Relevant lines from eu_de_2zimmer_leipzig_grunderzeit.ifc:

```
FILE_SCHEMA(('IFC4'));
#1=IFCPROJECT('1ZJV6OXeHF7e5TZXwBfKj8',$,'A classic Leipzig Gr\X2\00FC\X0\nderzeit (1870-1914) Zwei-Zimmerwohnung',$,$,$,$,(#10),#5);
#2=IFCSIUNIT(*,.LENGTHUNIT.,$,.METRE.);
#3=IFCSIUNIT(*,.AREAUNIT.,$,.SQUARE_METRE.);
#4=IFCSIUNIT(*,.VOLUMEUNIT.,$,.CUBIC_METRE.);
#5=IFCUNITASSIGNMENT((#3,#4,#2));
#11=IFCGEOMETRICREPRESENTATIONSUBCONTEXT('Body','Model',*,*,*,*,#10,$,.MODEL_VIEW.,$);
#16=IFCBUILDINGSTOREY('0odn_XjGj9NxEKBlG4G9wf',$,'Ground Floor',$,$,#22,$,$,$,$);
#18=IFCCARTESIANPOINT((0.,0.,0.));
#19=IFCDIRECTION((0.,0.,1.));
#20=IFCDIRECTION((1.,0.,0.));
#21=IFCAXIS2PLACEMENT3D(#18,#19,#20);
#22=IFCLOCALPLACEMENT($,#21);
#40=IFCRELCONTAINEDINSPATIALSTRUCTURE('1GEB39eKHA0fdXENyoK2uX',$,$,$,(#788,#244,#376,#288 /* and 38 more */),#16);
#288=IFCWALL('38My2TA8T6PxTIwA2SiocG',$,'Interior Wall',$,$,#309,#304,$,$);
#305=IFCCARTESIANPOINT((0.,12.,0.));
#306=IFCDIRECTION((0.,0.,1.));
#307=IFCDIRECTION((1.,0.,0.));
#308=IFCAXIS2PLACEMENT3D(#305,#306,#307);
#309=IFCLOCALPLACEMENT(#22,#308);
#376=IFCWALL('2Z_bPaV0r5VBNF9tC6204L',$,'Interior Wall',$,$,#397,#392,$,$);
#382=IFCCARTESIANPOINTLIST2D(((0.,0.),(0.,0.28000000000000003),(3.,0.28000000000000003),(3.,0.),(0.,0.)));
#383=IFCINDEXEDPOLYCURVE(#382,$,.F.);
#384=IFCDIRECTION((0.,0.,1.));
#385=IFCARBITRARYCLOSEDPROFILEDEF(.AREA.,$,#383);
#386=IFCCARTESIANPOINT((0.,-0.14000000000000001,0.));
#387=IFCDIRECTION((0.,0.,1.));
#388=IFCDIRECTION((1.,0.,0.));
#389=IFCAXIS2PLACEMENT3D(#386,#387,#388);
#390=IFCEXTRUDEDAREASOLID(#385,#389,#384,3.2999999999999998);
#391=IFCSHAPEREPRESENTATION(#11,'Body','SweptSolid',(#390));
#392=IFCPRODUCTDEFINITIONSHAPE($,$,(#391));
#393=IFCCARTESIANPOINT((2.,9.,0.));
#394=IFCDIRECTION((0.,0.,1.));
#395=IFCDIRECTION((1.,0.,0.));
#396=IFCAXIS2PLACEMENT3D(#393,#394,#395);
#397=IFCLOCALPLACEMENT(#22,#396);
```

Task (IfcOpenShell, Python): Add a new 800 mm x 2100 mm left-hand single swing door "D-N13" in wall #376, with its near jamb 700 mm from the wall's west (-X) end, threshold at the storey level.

```python
import numpy as np
import ifcopenshell
import ifcopenshell.api.feature
import ifcopenshell.api.geometry
import ifcopenshell.api.root
import ifcopenshell.api.spatial
import ifcopenshell.geom
import ifcopenshell.util.element
import ifcopenshell.util.placement
import ifcopenshell.util.representation
import ifcopenshell.util.shape
import ifcopenshell.util.unit

model = ifcopenshell.open("eu_de_2zimmer_leipzig_grunderzeit.ifc")
unit_scale = ifcopenshell.util.unit.calculate_unit_scale(model)
settings = ifcopenshell.geom.settings()


def volume(element):
    """Net volume in cubic metres, openings subtracted."""
    shape = ifcopenshell.geom.create_shape(settings, element)
    return ifcopenshell.util.shape.get_volume(shape.geometry)


wall = model.by_guid("2Z_bPaV0r5VBNF9tC6204L")
storey = ifcopenshell.util.element.get_container(wall, ifc_class="IfcBuildingStorey")
context = ifcopenshell.util.representation.get_context(model, "Model", "Body", "MODEL_VIEW")
before = volume(wall)

width, height, from_end, sill = 0.8, 2.1, 0.7, 0.0  # metres

# The wall runs along its own X axis, and the end named is its -X end.
wall_shape = ifcopenshell.geom.create_shape(settings, wall)
x, y, z = ifcopenshell.util.shape.get_vertices(wall_shape.geometry).T
start = x.min() + from_end
face, thickness = float(y.min()), float(y.max() - y.min())
wall_matrix = ifcopenshell.util.placement.get_local_placement(wall.ObjectPlacement)
level = ifcopenshell.util.placement.get_local_placement(storey.ObjectPlacement)[2, 3]


def in_wall(x, y):
    """Placement at x, y metres in the wall's axes, at sill height."""
    matrix = wall_matrix.copy()
    matrix[:, 3] = wall_matrix @ np.array([x / unit_scale, y / unit_scale, 0.0, 1.0])
    matrix[2, 3] = level + sill / unit_scale
    return matrix


# Opening: a box that overshoots both wall faces by 50 mm.
opening = ifcopenshell.api.root.create_entity(model, ifc_class="IfcOpeningElement", predefined_type="OPENING")
box = ifcopenshell.api.geometry.add_wall_representation(
    model, context=context, length=width, height=height, thickness=thickness + 0.1
)
ifcopenshell.api.geometry.assign_representation(model, product=opening, representation=box)
ifcopenshell.api.geometry.edit_object_placement(model, product=opening, matrix=in_wall(start, face - 0.05), is_si=False)
ifcopenshell.api.feature.add_feature(model, feature=opening, element=wall)

door = ifcopenshell.api.root.create_entity(model, ifc_class="IfcDoor", name="D-N13", predefined_type="DOOR")
door.OverallWidth, door.OverallHeight = width / unit_scale, height / unit_scale
door.OperationType = "SINGLE_SWING_LEFT"
body = ifcopenshell.api.geometry.add_door_representation(
    model,
    context=context,
    overall_width=door.OverallWidth,
    overall_height=door.OverallHeight,
    operation_type="SINGLE_SWING_LEFT",
    lining_properties={"LiningDepth": thickness / unit_scale, "ThresholdDepth": thickness / unit_scale},
)
ifcopenshell.api.geometry.assign_representation(model, product=door, representation=body)
ifcopenshell.api.spatial.assign_container(model, products=[door], relating_structure=storey)
ifcopenshell.api.feature.add_filling(model, opening=opening, element=door)

# The lining spans the wall, so the door starts at the wall face.
ifcopenshell.api.geometry.edit_object_placement(model, product=door, matrix=in_wall(start, face), is_si=False)

after = volume(wall)

print(f"wall volume {before:.3f} -> {after:.3f} m3")

model.write("eu_de_2zimmer_leipzig_grunderzeit-out.ifc")
```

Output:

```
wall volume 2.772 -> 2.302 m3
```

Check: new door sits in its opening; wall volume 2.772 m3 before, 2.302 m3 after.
